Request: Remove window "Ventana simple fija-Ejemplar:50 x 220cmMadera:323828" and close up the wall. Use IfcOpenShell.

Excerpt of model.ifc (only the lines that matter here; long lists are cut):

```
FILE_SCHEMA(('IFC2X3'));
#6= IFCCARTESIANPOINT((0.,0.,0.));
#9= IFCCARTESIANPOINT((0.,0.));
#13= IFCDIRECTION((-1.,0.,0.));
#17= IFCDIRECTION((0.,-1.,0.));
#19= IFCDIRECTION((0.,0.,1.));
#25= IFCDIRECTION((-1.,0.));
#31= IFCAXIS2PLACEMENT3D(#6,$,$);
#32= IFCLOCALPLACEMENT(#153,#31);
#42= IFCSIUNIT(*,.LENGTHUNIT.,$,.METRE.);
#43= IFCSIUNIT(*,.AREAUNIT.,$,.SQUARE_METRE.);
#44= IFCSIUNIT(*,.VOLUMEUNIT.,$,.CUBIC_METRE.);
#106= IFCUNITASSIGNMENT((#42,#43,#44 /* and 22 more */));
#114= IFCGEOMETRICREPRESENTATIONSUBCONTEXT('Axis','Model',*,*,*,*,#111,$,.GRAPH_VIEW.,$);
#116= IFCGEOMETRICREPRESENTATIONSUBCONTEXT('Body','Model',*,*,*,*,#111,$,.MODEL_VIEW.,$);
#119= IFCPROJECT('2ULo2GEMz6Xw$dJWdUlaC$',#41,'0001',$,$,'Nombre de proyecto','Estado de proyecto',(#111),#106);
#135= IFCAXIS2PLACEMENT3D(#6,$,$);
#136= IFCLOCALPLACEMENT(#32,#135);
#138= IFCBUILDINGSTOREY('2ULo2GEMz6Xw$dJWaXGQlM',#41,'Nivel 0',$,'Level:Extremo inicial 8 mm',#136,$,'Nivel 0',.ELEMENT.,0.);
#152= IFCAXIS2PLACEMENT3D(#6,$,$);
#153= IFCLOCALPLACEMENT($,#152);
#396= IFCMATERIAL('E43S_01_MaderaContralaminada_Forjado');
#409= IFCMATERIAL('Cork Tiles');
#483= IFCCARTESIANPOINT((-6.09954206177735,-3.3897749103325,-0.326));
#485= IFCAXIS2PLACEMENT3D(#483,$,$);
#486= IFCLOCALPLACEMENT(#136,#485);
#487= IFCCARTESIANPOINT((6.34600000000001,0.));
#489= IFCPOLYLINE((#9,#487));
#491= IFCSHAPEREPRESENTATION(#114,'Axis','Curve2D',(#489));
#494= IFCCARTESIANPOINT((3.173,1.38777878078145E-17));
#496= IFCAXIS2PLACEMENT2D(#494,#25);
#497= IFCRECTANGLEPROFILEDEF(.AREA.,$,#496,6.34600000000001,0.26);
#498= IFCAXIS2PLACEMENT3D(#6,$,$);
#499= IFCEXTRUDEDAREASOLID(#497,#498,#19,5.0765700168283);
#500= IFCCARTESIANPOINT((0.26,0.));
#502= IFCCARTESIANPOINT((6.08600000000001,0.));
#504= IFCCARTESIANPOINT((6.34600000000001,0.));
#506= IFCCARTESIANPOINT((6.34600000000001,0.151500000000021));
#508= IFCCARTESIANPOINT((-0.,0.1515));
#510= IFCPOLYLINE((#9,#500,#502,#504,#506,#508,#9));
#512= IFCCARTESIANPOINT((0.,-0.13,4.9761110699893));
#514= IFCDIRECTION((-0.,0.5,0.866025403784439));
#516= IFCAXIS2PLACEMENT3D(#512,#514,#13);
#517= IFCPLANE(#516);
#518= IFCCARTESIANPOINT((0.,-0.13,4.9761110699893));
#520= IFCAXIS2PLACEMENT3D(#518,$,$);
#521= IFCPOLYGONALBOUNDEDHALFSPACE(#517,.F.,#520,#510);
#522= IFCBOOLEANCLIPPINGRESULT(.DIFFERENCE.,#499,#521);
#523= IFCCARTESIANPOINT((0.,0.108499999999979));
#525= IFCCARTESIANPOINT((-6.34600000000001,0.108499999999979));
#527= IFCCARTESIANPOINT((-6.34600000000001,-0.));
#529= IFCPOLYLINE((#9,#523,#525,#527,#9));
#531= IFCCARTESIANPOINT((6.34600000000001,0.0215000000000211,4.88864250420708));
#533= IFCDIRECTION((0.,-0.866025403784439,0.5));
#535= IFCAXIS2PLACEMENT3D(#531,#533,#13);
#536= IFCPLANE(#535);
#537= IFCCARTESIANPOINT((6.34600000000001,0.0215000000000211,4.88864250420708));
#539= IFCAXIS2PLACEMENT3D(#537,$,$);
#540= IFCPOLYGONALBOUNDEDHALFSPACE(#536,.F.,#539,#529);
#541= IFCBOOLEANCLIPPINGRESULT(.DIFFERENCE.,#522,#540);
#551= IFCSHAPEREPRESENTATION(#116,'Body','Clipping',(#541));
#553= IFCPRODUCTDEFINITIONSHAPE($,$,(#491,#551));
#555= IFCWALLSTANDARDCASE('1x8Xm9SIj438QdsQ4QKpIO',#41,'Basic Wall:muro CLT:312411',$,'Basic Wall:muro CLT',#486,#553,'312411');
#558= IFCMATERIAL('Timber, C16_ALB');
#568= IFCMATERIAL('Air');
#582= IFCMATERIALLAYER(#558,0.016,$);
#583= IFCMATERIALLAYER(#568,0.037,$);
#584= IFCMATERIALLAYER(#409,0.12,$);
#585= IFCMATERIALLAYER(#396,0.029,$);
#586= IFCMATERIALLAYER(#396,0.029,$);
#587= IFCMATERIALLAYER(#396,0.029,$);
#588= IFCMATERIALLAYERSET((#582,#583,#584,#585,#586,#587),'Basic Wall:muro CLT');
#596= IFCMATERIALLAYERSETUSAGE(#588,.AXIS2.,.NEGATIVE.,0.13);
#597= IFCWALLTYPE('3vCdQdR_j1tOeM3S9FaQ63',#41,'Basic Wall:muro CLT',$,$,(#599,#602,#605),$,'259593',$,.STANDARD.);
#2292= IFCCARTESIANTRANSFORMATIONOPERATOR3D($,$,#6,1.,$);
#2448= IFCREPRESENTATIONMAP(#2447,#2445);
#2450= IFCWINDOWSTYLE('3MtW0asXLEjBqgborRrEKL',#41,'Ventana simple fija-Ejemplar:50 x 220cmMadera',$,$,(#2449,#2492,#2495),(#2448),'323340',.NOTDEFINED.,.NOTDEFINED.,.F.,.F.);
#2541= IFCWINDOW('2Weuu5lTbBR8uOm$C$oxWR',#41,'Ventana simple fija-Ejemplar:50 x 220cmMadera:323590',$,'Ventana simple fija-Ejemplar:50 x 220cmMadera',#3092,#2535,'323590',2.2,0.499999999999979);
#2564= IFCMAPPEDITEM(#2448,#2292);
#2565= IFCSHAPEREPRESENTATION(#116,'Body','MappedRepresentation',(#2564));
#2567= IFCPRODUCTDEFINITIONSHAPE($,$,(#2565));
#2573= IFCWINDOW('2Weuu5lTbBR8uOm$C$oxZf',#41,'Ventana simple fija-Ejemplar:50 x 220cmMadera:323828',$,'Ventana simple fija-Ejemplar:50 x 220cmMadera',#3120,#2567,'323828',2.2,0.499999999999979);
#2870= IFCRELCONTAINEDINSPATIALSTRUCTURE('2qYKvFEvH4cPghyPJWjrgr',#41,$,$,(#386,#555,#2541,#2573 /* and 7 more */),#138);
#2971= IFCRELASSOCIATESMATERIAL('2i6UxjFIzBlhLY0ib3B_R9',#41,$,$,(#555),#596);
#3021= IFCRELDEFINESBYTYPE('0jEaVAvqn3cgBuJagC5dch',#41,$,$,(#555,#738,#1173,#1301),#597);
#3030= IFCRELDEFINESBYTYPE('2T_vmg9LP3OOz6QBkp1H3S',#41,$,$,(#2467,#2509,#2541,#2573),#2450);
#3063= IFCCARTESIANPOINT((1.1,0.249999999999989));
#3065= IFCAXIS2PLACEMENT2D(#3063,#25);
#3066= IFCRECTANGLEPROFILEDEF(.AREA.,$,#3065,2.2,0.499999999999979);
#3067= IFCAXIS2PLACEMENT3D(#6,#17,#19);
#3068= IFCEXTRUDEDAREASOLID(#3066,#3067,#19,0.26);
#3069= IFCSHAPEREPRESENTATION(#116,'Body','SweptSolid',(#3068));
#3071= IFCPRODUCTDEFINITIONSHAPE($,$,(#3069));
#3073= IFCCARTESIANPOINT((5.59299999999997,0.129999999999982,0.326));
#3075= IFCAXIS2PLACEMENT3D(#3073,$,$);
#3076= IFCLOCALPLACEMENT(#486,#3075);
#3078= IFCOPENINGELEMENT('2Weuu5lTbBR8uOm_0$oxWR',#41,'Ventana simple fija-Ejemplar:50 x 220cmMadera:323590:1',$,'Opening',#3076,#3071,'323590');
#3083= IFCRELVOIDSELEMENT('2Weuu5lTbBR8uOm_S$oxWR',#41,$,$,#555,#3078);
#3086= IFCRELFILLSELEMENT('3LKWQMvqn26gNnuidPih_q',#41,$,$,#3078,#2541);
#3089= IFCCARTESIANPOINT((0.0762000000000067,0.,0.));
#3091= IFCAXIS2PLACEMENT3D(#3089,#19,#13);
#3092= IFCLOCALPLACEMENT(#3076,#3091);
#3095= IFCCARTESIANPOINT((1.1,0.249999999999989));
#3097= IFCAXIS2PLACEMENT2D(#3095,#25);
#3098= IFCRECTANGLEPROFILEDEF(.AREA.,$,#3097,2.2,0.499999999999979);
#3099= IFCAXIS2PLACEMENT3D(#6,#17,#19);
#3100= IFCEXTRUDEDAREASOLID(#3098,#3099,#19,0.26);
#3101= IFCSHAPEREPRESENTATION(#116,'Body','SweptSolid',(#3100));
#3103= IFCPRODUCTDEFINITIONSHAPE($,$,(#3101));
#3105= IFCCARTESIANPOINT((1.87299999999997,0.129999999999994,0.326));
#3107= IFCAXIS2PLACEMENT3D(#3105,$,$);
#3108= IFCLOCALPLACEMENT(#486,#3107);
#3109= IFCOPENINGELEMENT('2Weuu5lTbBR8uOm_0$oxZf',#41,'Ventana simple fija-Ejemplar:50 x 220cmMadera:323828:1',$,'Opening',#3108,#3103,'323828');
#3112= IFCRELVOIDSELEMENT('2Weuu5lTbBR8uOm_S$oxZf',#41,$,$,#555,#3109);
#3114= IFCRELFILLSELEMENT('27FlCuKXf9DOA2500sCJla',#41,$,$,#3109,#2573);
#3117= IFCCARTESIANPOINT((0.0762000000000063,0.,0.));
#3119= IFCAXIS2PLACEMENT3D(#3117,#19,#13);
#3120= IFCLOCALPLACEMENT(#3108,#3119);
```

```python
import ifcopenshell
import ifcopenshell.api.feature
import ifcopenshell.api.root
import ifcopenshell.geom
import ifcopenshell.util.shape

model = ifcopenshell.open("model.ifc")
settings = ifcopenshell.geom.settings()


def volume(element):
    """Net volume in cubic metres, openings subtracted."""
    shape = ifcopenshell.geom.create_shape(settings, element)
    return ifcopenshell.util.shape.get_volume(shape.geometry)


window = model.by_guid("2Weuu5lTbBR8uOm$C$oxZf")
opening = window.FillsVoids[0].RelatingOpeningElement
wall = opening.VoidsElements[0].RelatingBuildingElement
before = volume(wall)

ifcopenshell.api.root.remove_product(model, product=window)
ifcopenshell.api.feature.remove_feature(model, feature=opening)

after = volume(wall)

print(f"wall volume {before:.3f} -> {after:.3f} m3")

model.write("model_edited.ifc")
```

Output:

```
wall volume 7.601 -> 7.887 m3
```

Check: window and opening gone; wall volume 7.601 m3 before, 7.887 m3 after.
